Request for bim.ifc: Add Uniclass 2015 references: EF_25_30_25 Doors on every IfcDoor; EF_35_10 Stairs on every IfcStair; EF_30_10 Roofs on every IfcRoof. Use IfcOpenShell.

First a look at what the model holds.

```python
import ifcopenshell

model = ifcopenshell.open("bim.ifc")
print(model.schema)
print("classifications:", [c.Name for c in model.by_type("IfcClassification")])
for ifc_class in ("IfcDoor", "IfcRoof", "IfcStair", "IfcWall", "IfcWindow"):
    print(ifc_class, len(model.by_type(ifc_class)))
```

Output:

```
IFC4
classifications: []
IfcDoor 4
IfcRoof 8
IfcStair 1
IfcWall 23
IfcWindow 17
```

```python
import ifcopenshell
import ifcopenshell.api.classification

model = ifcopenshell.open("bim.ifc")

system = ifcopenshell.api.classification.add_classification(model, classification="Uniclass 2015")

codes = {
    "IfcDoor": ("EF_25_30_25", "Doors"),
    "IfcStair": ("EF_35_10", "Stairs"),
    "IfcRoof": ("EF_30_10", "Roofs"),
}
for ifc_class, (code, name) in codes.items():
    products = model.by_type(ifc_class)
    ifcopenshell.api.classification.add_reference(
        model, products=products, classification=system, identification=code, name=name
    )
    print(code, len(products))

model.write("bim_updated.ifc")
```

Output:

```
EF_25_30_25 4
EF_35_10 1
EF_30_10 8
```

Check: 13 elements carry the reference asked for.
